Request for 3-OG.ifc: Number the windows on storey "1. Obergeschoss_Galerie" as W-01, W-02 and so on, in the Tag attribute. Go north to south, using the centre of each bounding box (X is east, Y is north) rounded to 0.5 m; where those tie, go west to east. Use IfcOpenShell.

First a look at what the model holds.

```python
import ifcopenshell
import ifcopenshell.util.element
import ifcopenshell.util.placement

model = ifcopenshell.open("3-OG.ifc")
print(model.schema)
storey = next(s for s in model.by_type("IfcBuildingStorey") if s.Name == "1. Obergeschoss_Galerie")
windows = [e for e in ifcopenshell.util.element.get_decomposition(storey) if e.is_a("IfcWindow")]
for e in sorted(windows, key=lambda e: e.id()):
    origin = ifcopenshell.util.placement.get_local_placement(e.ObjectPlacement)[:3, 3]
    print(e.id(), e.Tag, e.Name, origin.round(2) + 0.0, sep=" | ")
```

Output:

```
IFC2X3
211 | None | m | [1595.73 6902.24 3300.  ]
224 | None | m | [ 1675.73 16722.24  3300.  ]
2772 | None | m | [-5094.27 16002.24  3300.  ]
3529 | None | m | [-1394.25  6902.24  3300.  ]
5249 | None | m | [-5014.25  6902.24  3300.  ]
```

```python
import ifcopenshell
import ifcopenshell.geom
import ifcopenshell.util.element
import ifcopenshell.util.shape

model = ifcopenshell.open("3-OG.ifc")
settings = ifcopenshell.geom.settings()
settings.set("use-world-coords", True)


def centre(element):
    shape = ifcopenshell.geom.create_shape(settings, element)
    return ifcopenshell.util.shape.get_bbox_centroid(shape.geometry)


storey = next(s for s in model.by_type("IfcBuildingStorey") if s.Name == "1. Obergeschoss_Galerie")
windows = [e for e in ifcopenshell.util.element.get_decomposition(storey) if e.is_a("IfcWindow")]

# Insertion points can sit at a corner or the storey origin, so sort by the geometry (in metres).
centres = {e: centre(e) for e in windows}
windows.sort(key=lambda e: (-round(centres[e][1] / 0.5), centres[e][0]))

for i, e in enumerate(windows, start=1):
    number = f"W-{i:02d}"
    e.Tag = number
    print(e.id(), number)

model.write("3-OG_updated.ifc")
```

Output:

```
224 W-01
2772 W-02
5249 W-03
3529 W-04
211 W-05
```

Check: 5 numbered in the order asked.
